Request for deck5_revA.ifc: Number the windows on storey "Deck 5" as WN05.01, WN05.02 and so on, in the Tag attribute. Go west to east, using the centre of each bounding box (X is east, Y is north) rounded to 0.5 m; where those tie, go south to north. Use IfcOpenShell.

First a look at what the model holds.

```python
import ifcopenshell
import ifcopenshell.util.element
import ifcopenshell.util.placement

model = ifcopenshell.open("deck5_revA.ifc")
print(model.schema)
storey = next(s for s in model.by_type("IfcBuildingStorey") if s.Name == "Deck 5")
windows = [e for e in ifcopenshell.util.element.get_decomposition(storey) if e.is_a("IfcWindow")]
for e in sorted(windows, key=lambda e: e.id()):
    origin = ifcopenshell.util.placement.get_local_placement(e.ObjectPlacement)[:3, 3]
    print(e.id(), e.Tag, e.Name, origin.round(2) + 0.0, sep=" | ")
```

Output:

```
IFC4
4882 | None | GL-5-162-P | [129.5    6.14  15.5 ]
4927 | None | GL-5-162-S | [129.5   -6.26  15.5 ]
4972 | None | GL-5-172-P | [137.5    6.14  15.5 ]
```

```python
import ifcopenshell
import ifcopenshell.geom
import ifcopenshell.util.element
import ifcopenshell.util.shape

model = ifcopenshell.open("deck5_revA.ifc")
settings = ifcopenshell.geom.settings()
settings.set("use-world-coords", True)


def centre(element):
    shape = ifcopenshell.geom.create_shape(settings, element)
    return ifcopenshell.util.shape.get_bbox_centroid(shape.geometry)


storey = next(s for s in model.by_type("IfcBuildingStorey") if s.Name == "Deck 5")
windows = [e for e in ifcopenshell.util.element.get_decomposition(storey) if e.is_a("IfcWindow")]

# Insertion points can sit at a corner or the storey origin, so sort by the geometry (in metres).
centres = {e: centre(e) for e in windows}
windows.sort(key=lambda e: (round(centres[e][0] / 0.5), centres[e][1]))

for i, e in enumerate(windows, start=1):
    number = f"WN05.{i:02d}"
    e.Tag = number
    print(e.id(), number)

model.write("deck5_revA_v2.ifc")
```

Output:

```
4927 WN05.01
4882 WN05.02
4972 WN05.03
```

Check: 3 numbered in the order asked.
